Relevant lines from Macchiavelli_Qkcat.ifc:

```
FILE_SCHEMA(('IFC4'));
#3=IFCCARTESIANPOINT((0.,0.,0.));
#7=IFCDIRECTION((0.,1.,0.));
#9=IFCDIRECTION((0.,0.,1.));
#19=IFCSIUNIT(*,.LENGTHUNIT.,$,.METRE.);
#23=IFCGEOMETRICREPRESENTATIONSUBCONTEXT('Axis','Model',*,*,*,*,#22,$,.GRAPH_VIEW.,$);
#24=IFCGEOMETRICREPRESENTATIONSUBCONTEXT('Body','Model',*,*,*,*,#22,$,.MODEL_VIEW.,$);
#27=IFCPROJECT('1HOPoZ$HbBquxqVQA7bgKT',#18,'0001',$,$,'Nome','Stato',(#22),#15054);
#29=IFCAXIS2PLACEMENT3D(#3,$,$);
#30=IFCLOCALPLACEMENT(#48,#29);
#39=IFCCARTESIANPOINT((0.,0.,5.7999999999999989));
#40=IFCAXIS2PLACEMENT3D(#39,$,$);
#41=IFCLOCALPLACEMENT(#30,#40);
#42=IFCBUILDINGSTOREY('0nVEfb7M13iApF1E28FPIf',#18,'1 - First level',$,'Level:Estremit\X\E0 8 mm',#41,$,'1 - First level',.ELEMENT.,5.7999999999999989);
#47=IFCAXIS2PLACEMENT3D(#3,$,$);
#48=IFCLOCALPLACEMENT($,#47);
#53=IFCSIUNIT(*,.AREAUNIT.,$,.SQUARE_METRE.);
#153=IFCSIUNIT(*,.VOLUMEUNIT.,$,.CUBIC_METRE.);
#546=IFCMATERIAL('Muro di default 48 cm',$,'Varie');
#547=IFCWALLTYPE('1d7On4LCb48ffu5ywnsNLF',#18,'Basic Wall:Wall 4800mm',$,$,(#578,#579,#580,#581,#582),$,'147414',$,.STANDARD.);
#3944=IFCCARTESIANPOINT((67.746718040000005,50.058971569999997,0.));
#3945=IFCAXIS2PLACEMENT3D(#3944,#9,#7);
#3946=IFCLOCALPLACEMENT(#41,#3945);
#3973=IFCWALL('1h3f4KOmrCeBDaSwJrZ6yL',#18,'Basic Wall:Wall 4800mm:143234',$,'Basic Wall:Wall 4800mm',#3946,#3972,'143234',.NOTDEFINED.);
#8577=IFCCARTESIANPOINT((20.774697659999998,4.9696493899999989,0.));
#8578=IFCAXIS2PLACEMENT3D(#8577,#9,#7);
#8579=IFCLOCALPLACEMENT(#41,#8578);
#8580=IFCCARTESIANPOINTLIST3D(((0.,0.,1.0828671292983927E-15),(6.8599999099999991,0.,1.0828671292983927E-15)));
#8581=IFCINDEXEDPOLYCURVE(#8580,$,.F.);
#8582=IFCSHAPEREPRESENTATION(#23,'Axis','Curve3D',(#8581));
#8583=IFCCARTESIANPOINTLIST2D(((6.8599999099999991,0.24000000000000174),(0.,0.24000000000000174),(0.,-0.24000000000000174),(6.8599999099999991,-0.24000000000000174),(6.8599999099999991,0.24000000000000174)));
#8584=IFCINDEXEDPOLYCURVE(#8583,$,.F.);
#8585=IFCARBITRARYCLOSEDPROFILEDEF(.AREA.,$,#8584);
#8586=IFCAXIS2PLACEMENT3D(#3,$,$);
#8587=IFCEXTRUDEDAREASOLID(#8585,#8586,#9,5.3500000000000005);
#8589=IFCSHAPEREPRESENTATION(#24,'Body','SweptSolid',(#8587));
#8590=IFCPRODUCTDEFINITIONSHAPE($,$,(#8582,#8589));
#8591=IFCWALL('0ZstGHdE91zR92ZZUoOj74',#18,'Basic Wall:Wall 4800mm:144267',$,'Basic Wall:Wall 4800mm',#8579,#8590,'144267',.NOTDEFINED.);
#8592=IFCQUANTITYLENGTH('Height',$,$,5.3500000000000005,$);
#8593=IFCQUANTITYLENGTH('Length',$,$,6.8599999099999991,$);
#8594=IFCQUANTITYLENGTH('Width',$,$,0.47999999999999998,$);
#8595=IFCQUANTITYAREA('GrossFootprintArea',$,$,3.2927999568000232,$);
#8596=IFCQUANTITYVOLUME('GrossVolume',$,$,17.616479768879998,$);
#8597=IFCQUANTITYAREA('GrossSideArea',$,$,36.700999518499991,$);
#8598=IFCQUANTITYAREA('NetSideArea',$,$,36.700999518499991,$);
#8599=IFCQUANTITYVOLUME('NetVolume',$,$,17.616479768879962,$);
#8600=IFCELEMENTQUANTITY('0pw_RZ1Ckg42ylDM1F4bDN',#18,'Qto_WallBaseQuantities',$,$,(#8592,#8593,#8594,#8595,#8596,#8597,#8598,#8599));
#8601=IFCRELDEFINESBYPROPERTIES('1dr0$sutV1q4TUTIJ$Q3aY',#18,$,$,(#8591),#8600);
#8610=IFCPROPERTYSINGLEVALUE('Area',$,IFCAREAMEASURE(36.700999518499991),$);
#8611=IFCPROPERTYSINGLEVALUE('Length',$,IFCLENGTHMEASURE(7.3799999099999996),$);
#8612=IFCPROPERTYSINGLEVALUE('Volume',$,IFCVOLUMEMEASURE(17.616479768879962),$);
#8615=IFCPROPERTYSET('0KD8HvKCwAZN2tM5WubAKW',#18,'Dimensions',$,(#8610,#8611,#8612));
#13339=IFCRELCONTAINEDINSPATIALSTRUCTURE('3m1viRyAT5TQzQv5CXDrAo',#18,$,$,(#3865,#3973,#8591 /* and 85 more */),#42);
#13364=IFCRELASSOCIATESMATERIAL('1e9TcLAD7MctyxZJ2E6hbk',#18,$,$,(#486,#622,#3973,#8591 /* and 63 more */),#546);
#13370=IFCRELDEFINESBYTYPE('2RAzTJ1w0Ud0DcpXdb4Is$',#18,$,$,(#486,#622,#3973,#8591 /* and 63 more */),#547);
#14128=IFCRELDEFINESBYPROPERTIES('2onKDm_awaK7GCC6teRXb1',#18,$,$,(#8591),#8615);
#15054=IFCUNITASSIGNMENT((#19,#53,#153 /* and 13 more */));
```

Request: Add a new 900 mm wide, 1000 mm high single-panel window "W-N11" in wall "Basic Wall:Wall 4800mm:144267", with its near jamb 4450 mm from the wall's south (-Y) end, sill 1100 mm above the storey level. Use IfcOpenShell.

```python
import numpy as np
import ifcopenshell
import ifcopenshell.api.feature
import ifcopenshell.api.geometry
import ifcopenshell.api.pset
import ifcopenshell.api.root
import ifcopenshell.api.spatial
import ifcopenshell.geom
import ifcopenshell.util.element
import ifcopenshell.util.placement
import ifcopenshell.util.representation
import ifcopenshell.util.shape
import ifcopenshell.util.unit

model = ifcopenshell.open("Macchiavelli_Qkcat.ifc")
unit_scale = ifcopenshell.util.unit.calculate_unit_scale(model)
area_scale = ifcopenshell.util.unit.calculate_unit_scale(model, "AREAUNIT")
volume_scale = ifcopenshell.util.unit.calculate_unit_scale(model, "VOLUMEUNIT")
settings = ifcopenshell.geom.settings()


def volume(element):
    """Net volume in cubic metres, openings subtracted."""
    shape = ifcopenshell.geom.create_shape(settings, element)
    return ifcopenshell.util.shape.get_volume(shape.geometry)


wall = model.by_guid("0ZstGHdE91zR92ZZUoOj74")
storey = ifcopenshell.util.element.get_container(wall, ifc_class="IfcBuildingStorey")
context = ifcopenshell.util.representation.get_context(model, "Model", "Body", "MODEL_VIEW")
before = volume(wall)

width, height, from_end, sill = 0.9, 1, 4.45, 1.1  # metres

# The wall runs along its own X axis, and the end named is its -X end.
wall_shape = ifcopenshell.geom.create_shape(settings, wall)
x, y, z = ifcopenshell.util.shape.get_vertices(wall_shape.geometry).T
start = x.min() + from_end
face, thickness = float(y.min()), float(y.max() - y.min())
wall_matrix = ifcopenshell.util.placement.get_local_placement(wall.ObjectPlacement)
level = ifcopenshell.util.placement.get_local_placement(storey.ObjectPlacement)[2, 3]


def in_wall(x, y):
    """Placement at x, y metres in the wall's axes, at sill height."""
    matrix = wall_matrix.copy()
    matrix[:, 3] = wall_matrix @ np.array([x / unit_scale, y / unit_scale, 0.0, 1.0])
    matrix[2, 3] = level + sill / unit_scale
    return matrix


# Opening: a box that overshoots both wall faces by 50 mm.
opening = ifcopenshell.api.root.create_entity(model, ifc_class="IfcOpeningElement", predefined_type="OPENING")
box = ifcopenshell.api.geometry.add_wall_representation(
    model, context=context, length=width, height=height, thickness=thickness + 0.1
)
ifcopenshell.api.geometry.assign_representation(model, product=opening, representation=box)
ifcopenshell.api.geometry.edit_object_placement(model, product=opening, matrix=in_wall(start, face - 0.05), is_si=False)
ifcopenshell.api.feature.add_feature(model, feature=opening, element=wall)

window = ifcopenshell.api.root.create_entity(model, ifc_class="IfcWindow", name="W-N11", predefined_type="WINDOW")
window.OverallWidth, window.OverallHeight = width / unit_scale, height / unit_scale
window.PartitioningType = "SINGLE_PANEL"
body = ifcopenshell.api.geometry.add_window_representation(
    model,
    context=context,
    overall_width=window.OverallWidth,
    overall_height=window.OverallHeight,
    partition_type="SINGLE_PANEL",
)
ifcopenshell.api.geometry.assign_representation(model, product=window, representation=body)
ifcopenshell.api.spatial.assign_container(model, products=[window], relating_structure=storey)
ifcopenshell.api.feature.add_filling(model, opening=opening, element=window)

# Centre the window in the wall's thickness.
ifcopenshell.api.geometry.edit_object_placement(model, product=window, matrix=in_wall(start, face), is_si=False)
window_shape = ifcopenshell.geom.create_shape(settings, window)
depth = ifcopenshell.util.shape.get_vertices(window_shape.geometry)[:, 1]
offset = face + thickness / 2 - (depth.min() + depth.max()) / 2
ifcopenshell.api.geometry.edit_object_placement(model, product=window, matrix=in_wall(start, offset), is_si=False)

after = volume(wall)

# Update the wall's stored quantities.
qto = model.by_id(ifcopenshell.util.element.get_pset(wall, "Qto_WallBaseQuantities", should_inherit=False)["id"])
ifcopenshell.api.pset.edit_qto(model, qto=qto, properties={
    "NetSideArea": after / thickness / area_scale,
    "NetVolume": after / volume_scale,
})
pset = model.by_id(ifcopenshell.util.element.get_pset(wall, "Dimensions", should_inherit=False)["id"])
ifcopenshell.api.pset.edit_pset(model, pset=pset, properties={
    "Area": model.create_entity("IfcAreaMeasure", after / thickness / area_scale),
    "Volume": model.create_entity("IfcVolumeMeasure", after / volume_scale),
})

print(f"wall volume {before:.3f} -> {after:.3f} m3")

model.write("Macchiavelli_Qkcat-out.ifc")
```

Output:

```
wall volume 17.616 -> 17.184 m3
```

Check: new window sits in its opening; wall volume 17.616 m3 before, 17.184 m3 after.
